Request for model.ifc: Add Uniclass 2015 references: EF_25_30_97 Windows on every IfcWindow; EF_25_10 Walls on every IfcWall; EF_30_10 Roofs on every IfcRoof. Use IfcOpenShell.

First a look at what the model holds.

```python
import ifcopenshell

model = ifcopenshell.open("model.ifc")
print(model.schema)
print("classifications:", [c.Name for c in model.by_type("IfcClassification")])
for ifc_class in ("IfcDoor", "IfcRoof", "IfcStair", "IfcWall", "IfcWindow"):
    print(ifc_class, len(model.by_type(ifc_class)))
```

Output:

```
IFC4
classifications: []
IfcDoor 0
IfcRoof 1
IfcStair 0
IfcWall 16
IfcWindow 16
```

```python
import ifcopenshell
import ifcopenshell.api.classification

model = ifcopenshell.open("model.ifc")

system = ifcopenshell.api.classification.add_classification(model, classification="Uniclass 2015")

codes = {
    "IfcWindow": ("EF_25_30_97", "Windows"),
    "IfcWall": ("EF_25_10", "Walls"),
    "IfcRoof": ("EF_30_10", "Roofs"),
}
for ifc_class, (code, name) in codes.items():
    products = model.by_type(ifc_class)
    ifcopenshell.api.classification.add_reference(
        model, products=products, classification=system, identification=code, name=name
    )
    print(code, len(products))

model.write("model_edited.ifc")
```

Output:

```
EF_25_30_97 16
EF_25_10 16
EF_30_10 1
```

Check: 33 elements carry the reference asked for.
